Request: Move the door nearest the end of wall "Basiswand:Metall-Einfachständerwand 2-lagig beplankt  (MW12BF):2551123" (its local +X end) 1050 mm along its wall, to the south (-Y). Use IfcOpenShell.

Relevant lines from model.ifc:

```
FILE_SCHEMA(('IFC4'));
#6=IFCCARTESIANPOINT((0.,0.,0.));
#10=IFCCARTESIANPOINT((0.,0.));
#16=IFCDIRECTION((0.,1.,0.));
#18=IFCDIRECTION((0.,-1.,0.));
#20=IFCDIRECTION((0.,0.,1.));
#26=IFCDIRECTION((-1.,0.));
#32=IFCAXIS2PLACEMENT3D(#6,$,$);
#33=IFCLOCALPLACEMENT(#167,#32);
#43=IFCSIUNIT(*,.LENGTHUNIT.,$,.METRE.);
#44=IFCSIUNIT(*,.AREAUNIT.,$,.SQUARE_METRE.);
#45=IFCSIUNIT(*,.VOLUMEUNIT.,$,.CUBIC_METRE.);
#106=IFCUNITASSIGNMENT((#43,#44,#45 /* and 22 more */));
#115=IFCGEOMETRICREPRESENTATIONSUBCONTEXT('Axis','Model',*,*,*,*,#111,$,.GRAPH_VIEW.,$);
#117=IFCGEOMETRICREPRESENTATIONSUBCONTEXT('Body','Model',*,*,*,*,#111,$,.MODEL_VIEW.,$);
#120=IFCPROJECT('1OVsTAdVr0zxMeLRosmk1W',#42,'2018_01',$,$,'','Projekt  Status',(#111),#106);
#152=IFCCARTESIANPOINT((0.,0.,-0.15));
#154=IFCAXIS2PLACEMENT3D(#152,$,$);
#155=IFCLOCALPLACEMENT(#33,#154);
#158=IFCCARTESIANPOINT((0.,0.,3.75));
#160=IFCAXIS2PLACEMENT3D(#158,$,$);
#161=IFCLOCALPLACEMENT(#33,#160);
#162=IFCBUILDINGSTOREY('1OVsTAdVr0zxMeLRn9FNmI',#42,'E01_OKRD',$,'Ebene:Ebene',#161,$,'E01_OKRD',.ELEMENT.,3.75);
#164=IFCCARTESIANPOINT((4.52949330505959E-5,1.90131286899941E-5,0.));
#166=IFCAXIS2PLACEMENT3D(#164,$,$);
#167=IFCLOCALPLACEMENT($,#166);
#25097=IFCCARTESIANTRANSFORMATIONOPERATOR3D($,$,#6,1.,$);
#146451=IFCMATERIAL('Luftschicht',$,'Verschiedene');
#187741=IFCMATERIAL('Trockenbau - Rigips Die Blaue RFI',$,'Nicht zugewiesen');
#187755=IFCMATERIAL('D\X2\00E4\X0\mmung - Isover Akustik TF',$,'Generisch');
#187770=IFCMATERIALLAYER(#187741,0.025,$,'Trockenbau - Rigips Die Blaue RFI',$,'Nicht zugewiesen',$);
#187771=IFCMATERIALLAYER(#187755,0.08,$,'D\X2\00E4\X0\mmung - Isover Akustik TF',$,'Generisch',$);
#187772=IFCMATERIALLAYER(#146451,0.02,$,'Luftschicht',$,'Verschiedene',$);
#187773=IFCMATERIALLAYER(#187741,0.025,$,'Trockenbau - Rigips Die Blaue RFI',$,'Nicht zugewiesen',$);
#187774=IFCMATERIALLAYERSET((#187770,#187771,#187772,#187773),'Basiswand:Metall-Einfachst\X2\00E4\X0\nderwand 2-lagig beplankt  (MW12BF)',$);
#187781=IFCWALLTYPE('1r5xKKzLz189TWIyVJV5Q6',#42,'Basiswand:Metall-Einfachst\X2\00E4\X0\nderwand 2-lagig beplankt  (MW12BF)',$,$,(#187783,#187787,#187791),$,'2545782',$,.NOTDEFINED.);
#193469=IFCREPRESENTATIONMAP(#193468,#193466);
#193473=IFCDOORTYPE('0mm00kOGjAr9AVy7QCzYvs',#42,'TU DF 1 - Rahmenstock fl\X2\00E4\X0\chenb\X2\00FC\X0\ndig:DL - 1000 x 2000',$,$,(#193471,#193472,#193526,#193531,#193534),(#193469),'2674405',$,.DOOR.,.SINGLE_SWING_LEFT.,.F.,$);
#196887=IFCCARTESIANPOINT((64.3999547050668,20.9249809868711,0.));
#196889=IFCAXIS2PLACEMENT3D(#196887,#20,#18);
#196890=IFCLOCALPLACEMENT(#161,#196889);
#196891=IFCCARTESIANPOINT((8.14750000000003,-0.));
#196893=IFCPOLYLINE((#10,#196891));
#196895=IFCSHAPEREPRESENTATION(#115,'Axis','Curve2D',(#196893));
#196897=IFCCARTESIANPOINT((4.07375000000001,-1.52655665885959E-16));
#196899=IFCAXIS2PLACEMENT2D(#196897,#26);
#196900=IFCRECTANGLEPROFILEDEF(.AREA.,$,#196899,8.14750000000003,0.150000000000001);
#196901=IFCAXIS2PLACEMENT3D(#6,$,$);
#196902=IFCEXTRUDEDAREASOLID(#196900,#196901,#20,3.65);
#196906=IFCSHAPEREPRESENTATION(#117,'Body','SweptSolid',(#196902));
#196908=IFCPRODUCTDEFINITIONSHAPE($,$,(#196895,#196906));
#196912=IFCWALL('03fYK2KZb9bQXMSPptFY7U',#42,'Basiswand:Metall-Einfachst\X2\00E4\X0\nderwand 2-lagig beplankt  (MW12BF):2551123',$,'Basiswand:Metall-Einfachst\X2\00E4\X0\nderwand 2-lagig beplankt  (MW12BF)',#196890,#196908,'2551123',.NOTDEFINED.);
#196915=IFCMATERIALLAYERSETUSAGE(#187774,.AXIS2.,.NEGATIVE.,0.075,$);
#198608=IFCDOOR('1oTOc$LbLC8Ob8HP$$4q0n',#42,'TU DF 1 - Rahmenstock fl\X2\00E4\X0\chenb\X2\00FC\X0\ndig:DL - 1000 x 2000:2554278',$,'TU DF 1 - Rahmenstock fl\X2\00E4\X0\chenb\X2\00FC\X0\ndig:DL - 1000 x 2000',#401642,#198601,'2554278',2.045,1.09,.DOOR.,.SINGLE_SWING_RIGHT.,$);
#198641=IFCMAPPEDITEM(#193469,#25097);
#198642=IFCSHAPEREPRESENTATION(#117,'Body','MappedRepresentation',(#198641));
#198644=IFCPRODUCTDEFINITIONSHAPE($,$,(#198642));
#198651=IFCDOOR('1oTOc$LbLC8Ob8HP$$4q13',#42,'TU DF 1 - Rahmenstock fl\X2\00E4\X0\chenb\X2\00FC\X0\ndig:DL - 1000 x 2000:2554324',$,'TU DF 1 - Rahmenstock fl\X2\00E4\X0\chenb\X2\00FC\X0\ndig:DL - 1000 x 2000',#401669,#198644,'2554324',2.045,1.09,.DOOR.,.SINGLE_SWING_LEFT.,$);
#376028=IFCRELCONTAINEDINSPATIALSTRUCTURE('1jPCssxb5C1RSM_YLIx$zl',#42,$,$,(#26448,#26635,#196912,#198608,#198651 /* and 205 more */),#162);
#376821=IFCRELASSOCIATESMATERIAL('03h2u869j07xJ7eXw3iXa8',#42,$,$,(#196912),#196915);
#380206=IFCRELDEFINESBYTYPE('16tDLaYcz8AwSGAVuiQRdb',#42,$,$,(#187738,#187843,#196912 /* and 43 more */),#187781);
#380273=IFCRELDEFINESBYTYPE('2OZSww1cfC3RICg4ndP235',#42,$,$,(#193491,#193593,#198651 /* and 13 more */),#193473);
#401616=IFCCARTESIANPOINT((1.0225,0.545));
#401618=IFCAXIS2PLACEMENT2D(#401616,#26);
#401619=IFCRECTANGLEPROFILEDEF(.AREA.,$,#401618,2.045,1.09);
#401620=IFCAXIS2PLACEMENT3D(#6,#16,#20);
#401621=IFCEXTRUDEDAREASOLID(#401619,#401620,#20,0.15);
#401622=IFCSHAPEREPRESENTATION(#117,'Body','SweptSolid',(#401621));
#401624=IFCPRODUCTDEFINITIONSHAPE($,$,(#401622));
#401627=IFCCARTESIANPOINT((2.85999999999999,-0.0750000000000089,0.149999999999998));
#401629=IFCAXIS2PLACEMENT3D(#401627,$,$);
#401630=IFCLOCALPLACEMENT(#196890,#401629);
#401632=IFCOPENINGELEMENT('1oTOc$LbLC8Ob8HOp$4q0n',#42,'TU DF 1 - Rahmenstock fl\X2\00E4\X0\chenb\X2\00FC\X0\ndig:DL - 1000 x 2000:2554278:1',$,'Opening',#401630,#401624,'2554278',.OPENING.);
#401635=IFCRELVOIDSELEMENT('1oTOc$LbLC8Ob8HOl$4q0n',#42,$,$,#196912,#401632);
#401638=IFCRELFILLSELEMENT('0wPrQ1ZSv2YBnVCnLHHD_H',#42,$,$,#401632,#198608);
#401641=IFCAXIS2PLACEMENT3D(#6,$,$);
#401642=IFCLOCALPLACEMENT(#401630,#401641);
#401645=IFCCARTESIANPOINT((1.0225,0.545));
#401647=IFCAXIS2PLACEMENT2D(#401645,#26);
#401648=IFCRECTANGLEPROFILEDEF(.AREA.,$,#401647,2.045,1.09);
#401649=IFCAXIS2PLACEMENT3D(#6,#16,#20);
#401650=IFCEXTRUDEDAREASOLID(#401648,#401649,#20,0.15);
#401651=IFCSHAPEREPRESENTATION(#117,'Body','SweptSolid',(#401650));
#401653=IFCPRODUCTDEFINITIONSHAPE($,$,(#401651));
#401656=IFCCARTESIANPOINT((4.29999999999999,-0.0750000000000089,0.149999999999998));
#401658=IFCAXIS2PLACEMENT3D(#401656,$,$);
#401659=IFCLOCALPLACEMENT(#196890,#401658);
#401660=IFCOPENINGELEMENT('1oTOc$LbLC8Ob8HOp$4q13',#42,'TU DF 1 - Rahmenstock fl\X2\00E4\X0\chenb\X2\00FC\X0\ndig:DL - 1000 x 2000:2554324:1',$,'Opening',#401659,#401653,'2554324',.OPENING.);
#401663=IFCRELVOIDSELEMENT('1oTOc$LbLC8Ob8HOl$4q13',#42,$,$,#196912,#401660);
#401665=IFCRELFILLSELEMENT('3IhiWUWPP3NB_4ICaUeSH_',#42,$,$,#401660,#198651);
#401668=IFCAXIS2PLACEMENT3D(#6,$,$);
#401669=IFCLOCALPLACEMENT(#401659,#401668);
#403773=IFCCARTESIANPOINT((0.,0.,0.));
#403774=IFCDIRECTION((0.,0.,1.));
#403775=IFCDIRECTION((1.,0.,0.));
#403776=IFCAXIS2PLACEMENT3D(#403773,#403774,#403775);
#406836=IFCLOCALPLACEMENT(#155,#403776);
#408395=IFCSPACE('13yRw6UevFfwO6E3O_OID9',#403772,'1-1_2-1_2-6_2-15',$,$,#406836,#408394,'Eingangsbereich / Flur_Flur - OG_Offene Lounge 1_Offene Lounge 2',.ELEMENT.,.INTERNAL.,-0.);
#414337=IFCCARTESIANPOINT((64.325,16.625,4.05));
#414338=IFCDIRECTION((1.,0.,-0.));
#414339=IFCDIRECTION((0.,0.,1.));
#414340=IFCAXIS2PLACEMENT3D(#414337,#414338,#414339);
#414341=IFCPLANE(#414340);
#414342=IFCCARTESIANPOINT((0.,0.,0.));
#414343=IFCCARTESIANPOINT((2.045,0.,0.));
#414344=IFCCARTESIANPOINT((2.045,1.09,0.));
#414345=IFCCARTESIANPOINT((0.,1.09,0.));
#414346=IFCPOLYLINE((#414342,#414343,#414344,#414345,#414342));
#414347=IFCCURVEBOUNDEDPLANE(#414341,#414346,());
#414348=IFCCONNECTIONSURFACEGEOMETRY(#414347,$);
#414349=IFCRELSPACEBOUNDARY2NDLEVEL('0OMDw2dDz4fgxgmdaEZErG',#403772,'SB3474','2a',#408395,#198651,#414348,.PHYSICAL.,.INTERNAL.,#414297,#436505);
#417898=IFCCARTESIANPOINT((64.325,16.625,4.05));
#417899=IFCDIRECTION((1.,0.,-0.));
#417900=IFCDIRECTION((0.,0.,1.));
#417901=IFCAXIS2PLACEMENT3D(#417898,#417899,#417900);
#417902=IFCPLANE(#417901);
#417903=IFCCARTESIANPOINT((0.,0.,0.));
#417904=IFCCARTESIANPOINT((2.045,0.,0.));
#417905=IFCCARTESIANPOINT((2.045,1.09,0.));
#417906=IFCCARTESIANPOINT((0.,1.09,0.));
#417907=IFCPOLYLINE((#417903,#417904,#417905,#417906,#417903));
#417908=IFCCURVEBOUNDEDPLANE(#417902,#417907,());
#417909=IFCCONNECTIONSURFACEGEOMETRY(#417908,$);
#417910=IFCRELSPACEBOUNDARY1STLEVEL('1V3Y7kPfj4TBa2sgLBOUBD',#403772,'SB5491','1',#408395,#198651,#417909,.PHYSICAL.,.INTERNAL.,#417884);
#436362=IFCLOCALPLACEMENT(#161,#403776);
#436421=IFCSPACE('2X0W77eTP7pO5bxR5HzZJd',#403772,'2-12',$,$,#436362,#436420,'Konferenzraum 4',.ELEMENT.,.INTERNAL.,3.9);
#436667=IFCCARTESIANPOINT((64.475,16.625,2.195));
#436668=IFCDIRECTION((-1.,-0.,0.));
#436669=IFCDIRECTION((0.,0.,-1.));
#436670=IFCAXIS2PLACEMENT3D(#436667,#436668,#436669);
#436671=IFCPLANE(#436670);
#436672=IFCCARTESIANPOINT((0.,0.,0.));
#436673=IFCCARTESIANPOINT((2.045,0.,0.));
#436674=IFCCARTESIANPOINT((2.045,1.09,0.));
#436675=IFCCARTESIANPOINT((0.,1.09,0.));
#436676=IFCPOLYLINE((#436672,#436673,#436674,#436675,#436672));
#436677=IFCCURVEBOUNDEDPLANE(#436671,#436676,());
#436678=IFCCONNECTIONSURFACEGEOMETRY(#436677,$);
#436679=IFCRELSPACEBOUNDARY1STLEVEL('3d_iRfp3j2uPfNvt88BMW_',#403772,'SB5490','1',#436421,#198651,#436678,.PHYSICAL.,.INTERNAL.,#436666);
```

```python
import numpy as np
import ifcopenshell
import ifcopenshell.api.geometry
import ifcopenshell.util.placement
import ifcopenshell.util.unit

model = ifcopenshell.open("model.ifc")
unit_scale = ifcopenshell.util.unit.calculate_unit_scale(model)

door = model.by_guid("1oTOc$LbLC8Ob8HP$$4q13")
opening = door.FillsVoids[0].RelatingOpeningElement
wall = opening.VoidsElements[0].RelatingBuildingElement

wall_matrix = ifcopenshell.util.placement.get_local_placement(wall.ObjectPlacement)
shift = wall_matrix[:3, 0] * 1.05 / unit_scale
before = ifcopenshell.util.placement.get_local_placement(door.ObjectPlacement)[:3, 3].copy()

# The door is placed relative to its opening, so it follows when the opening moves.
matrix = ifcopenshell.util.placement.get_local_placement(opening.ObjectPlacement)
matrix[:3, 3] += shift
ifcopenshell.api.geometry.edit_object_placement(
    model, product=opening, matrix=matrix, is_si=False, should_transform_children=True
)

# Space boundary surfaces are stored in each space's coordinates; move them too.
for rel in door.ProvidesBoundaries:
    if not rel.ConnectionGeometry:
        continue
    surface = rel.ConnectionGeometry.SurfaceOnRelatingElement.BasisSurface
    space_matrix = ifcopenshell.util.placement.get_local_placement(rel.RelatingSpace.ObjectPlacement)
    point = np.array(surface.Position.Location.Coordinates) + space_matrix[:3, :3].T @ shift
    surface.Position = model.createIfcAxis2Placement3D(
        model.createIfcCartesianPoint(point.tolist()), surface.Position.Axis, surface.Position.RefDirection
    )

after = ifcopenshell.util.placement.get_local_placement(door.ObjectPlacement)[:3, 3]
print("door moved by", (after - before).round(3) + 0.0)

model.write("model-out.ifc")
```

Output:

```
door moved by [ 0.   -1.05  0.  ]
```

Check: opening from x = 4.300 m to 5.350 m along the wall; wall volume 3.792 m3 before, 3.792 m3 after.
